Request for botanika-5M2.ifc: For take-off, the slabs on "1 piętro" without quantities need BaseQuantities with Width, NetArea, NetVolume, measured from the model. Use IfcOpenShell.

First a look at what the model holds.

```python
import ifcopenshell
import ifcopenshell.util.element
import ifcopenshell.util.unit

model = ifcopenshell.open("botanika-5M2.ifc")
print(model.schema)
for unit_type in ("LENGTHUNIT", "AREAUNIT", "VOLUMEUNIT"):
    print(unit_type, ifcopenshell.util.unit.calculate_unit_scale(model, unit_type))
storey = next(s for s in model.by_type("IfcBuildingStorey") if s.Name == "1 piętro")
slabs = [e for e in ifcopenshell.util.element.get_decomposition(storey) if e.is_a("IfcSlab")]
for e in sorted(slabs, key=lambda e: e.id()):
    print(e.id(), e.is_a(), e.Name, list(ifcopenshell.util.element.get_psets(e, qtos_only=True)), sep=" | ")
```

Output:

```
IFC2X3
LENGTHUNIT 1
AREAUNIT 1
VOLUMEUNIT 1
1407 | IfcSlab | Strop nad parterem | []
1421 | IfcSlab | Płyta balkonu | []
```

```python
import ifcopenshell
import ifcopenshell.api.pset
import ifcopenshell.geom
import ifcopenshell.util.element
import ifcopenshell.util.shape
import ifcopenshell.util.unit

model = ifcopenshell.open("botanika-5M2.ifc")
unit_scale = ifcopenshell.util.unit.calculate_unit_scale(model)
area_scale = ifcopenshell.util.unit.calculate_unit_scale(model, "AREAUNIT")
volume_scale = ifcopenshell.util.unit.calculate_unit_scale(model, "VOLUMEUNIT")
settings = ifcopenshell.geom.settings()

storey = next(s for s in model.by_type("IfcBuildingStorey") if s.Name == "1 piętro")
slabs = [e for e in ifcopenshell.util.element.get_decomposition(storey) if e.is_a("IfcSlab")]

for e in sorted(slabs, key=lambda e: e.id()):
    if ifcopenshell.util.element.get_psets(e, qtos_only=True, should_inherit=False):
        continue
    # Geometry comes back in metres, in the element's own axes.
    shape = ifcopenshell.geom.create_shape(settings, e)
    values = {
        "Width": ifcopenshell.util.shape.get_z(shape.geometry) / unit_scale,
        "NetArea": ifcopenshell.util.shape.get_footprint_area(shape.geometry) / area_scale,
        "NetVolume": ifcopenshell.util.shape.get_volume(shape.geometry) / volume_scale,
    }
    qto = ifcopenshell.api.pset.add_qto(model, product=e, name="BaseQuantities")
    ifcopenshell.api.pset.edit_qto(model, qto=qto, properties=values)
    print(e.id(), {k: round(v, 3) for k, v in values.items()})

model.write("botanika-5M2_edited.ifc")
```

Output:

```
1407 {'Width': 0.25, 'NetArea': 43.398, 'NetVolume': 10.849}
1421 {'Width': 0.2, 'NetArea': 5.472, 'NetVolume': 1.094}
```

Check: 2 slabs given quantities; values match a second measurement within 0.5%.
